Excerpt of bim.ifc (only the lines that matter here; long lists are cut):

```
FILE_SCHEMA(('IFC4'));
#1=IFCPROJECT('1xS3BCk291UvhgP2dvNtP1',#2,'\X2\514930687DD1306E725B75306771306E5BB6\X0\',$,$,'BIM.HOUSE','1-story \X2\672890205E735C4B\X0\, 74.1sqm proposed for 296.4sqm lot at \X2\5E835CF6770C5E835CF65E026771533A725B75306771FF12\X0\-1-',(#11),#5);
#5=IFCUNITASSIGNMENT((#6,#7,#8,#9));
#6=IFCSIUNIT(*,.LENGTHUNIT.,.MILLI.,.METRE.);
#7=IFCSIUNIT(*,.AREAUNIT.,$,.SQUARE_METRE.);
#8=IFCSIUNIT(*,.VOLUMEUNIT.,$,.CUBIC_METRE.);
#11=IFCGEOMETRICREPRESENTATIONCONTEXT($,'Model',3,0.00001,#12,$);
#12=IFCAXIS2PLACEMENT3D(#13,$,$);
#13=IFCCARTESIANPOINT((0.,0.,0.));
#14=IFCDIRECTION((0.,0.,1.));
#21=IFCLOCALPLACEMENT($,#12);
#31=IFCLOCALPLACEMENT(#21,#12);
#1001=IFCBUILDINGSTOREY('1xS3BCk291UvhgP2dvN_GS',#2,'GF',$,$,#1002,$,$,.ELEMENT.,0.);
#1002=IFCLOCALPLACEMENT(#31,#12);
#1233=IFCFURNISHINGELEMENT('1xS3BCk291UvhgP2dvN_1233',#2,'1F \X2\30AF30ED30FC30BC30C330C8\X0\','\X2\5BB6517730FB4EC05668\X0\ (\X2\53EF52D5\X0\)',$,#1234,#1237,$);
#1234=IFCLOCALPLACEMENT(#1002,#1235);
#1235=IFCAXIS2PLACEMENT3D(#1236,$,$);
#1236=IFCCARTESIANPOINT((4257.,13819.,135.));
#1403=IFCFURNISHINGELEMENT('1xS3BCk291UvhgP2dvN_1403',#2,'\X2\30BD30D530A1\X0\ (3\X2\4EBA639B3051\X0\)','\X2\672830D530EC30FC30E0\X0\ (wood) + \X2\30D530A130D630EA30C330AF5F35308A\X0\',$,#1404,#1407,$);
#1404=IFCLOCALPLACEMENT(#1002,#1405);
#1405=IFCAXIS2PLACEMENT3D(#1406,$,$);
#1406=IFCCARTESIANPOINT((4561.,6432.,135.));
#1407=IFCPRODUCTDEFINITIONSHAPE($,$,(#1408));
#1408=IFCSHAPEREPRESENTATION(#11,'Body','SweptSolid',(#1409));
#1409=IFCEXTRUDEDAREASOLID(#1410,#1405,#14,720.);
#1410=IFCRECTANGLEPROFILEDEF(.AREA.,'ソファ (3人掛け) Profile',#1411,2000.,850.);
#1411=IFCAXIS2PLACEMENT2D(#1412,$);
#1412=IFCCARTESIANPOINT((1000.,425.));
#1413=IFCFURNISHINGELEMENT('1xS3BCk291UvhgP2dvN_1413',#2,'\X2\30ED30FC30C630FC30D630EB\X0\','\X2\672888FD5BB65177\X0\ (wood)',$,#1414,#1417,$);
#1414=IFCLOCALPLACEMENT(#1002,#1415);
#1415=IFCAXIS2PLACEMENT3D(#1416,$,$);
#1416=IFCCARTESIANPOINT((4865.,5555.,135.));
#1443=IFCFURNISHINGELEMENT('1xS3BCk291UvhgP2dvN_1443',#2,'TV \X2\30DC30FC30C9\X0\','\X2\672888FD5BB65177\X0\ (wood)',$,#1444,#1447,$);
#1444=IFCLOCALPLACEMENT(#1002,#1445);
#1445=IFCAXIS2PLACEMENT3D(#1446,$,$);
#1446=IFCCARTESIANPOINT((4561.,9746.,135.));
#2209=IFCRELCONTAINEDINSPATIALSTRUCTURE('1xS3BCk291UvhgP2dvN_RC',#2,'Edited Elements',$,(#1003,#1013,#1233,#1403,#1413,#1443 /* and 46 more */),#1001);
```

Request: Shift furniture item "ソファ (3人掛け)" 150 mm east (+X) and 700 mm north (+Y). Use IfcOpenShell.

```python
import ifcopenshell
import ifcopenshell.api.geometry
import ifcopenshell.util.placement
import ifcopenshell.util.unit

model = ifcopenshell.open("bim.ifc")
unit_scale = ifcopenshell.util.unit.calculate_unit_scale(model)

item = model.by_id(1403)
matrix = ifcopenshell.util.placement.get_local_placement(item.ObjectPlacement)
matrix[0, 3] += 0.15 / unit_scale
matrix[1, 3] += 0.7 / unit_scale
ifcopenshell.api.geometry.edit_object_placement(model, product=item, matrix=matrix, is_si=False)

print(ifcopenshell.util.placement.get_local_placement(item.ObjectPlacement).round(3) + 0.0)

model.write("bim_edited.ifc")
```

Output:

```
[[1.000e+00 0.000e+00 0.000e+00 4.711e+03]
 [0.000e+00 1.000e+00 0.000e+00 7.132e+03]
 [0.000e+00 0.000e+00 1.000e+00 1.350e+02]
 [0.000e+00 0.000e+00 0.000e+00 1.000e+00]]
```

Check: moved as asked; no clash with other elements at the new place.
